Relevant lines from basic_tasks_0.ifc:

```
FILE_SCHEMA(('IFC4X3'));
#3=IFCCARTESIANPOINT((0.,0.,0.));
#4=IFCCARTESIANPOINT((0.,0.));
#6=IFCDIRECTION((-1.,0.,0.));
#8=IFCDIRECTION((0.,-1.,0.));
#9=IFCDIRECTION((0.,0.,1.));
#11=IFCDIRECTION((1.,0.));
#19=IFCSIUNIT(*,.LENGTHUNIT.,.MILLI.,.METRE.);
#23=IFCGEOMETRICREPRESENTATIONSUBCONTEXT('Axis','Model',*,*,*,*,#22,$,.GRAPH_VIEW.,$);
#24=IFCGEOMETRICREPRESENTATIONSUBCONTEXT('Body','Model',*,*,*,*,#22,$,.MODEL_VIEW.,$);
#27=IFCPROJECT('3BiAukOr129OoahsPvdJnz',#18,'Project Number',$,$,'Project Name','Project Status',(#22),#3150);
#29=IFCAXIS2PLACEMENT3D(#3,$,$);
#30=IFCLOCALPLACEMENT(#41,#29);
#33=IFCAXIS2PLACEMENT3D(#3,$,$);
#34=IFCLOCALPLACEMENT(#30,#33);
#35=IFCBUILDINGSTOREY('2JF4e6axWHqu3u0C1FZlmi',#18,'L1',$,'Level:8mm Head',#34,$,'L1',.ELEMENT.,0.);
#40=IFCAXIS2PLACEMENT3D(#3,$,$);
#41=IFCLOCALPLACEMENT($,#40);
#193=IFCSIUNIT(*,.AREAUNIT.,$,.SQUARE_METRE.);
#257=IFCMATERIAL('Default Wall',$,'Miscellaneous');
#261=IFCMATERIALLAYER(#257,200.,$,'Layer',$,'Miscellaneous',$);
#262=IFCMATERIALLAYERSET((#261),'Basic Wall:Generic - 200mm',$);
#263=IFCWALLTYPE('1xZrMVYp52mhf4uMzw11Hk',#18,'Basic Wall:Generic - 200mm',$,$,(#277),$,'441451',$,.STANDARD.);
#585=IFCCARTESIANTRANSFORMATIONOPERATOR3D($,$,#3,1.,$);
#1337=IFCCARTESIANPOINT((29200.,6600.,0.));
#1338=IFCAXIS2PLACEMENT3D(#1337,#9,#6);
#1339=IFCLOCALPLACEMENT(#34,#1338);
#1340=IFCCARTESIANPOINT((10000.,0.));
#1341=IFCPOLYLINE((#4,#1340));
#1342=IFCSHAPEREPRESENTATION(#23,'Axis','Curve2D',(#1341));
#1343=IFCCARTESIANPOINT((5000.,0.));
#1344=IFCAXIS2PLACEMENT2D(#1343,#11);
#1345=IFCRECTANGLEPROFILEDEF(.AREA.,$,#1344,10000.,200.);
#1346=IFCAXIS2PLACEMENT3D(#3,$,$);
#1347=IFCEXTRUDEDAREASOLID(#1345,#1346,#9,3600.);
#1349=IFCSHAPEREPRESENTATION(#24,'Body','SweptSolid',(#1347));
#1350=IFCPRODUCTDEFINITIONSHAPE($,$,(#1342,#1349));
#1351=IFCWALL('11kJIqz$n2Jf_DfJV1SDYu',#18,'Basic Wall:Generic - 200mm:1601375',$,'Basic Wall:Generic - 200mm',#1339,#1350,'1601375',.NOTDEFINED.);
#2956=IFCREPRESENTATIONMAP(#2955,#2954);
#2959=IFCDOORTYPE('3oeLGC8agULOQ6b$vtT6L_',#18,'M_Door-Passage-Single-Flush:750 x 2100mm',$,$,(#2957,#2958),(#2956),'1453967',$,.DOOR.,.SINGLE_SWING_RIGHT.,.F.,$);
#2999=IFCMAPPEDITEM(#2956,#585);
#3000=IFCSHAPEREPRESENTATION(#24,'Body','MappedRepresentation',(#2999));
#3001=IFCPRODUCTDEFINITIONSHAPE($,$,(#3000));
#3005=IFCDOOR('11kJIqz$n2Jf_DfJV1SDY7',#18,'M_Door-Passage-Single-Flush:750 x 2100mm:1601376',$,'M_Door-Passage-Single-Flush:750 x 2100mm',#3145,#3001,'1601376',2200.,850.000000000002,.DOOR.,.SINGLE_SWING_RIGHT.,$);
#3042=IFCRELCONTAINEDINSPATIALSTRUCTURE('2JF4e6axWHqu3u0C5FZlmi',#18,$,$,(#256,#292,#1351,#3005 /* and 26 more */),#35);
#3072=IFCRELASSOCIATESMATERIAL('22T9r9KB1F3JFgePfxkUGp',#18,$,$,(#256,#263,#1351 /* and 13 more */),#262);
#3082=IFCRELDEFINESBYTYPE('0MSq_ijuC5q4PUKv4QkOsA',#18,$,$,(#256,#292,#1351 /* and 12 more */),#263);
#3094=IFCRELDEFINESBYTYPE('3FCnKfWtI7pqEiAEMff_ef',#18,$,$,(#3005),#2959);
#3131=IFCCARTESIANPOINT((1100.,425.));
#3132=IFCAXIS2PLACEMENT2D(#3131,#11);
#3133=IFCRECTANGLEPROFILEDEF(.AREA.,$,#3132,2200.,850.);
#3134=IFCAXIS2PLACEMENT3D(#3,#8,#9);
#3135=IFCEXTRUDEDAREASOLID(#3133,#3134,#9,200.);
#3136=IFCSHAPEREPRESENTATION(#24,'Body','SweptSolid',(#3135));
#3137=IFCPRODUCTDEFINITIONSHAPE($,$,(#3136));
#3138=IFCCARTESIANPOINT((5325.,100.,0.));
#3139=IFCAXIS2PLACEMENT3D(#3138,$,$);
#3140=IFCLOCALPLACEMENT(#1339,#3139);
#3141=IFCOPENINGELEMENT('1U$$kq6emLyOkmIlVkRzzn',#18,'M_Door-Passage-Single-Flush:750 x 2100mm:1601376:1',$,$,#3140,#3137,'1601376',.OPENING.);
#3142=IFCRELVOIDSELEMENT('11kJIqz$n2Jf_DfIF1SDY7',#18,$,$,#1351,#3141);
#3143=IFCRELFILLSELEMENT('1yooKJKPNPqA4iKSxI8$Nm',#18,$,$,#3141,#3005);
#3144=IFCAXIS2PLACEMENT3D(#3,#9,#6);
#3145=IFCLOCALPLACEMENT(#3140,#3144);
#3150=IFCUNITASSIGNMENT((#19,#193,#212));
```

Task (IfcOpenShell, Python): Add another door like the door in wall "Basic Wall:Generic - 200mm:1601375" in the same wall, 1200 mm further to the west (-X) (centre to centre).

```python
import ifcopenshell
import ifcopenshell.api.feature
import ifcopenshell.api.geometry
import ifcopenshell.api.root
import ifcopenshell.geom
import ifcopenshell.util.element
import ifcopenshell.util.placement
import ifcopenshell.util.shape
import ifcopenshell.util.unit

model = ifcopenshell.open("basic_tasks_0.ifc")
unit_scale = ifcopenshell.util.unit.calculate_unit_scale(model)
settings = ifcopenshell.geom.settings()


def volume(element):
    """Net volume in cubic metres, openings subtracted."""
    shape = ifcopenshell.geom.create_shape(settings, element)
    return ifcopenshell.util.shape.get_volume(shape.geometry)


def reuse_history(source, copy):
    """copy_class also copies each property set's owner history, people and application; keep the originals."""
    for rel in copy.IsDefinedBy:
        if rel.is_a("IfcRelDefinesByProperties") and (history := rel.RelatingPropertyDefinition.OwnerHistory):
            rel.RelatingPropertyDefinition.OwnerHistory = source.OwnerHistory
            ifcopenshell.util.element.remove_deep2(model, history)


door = model.by_guid("11kJIqz$n2Jf_DfJV1SDY7")
opening = door.FillsVoids[0].RelatingOpeningElement
wall = opening.VoidsElements[0].RelatingBuildingElement
before = volume(wall)
shift = ifcopenshell.util.placement.get_local_placement(wall.ObjectPlacement)[:3, 0] * 1.2 / unit_scale

# copy_class copies the void relationship, type, container and properties, but no geometry.
new_opening = ifcopenshell.api.root.copy_class(model, product=opening)
new_opening.Representation = ifcopenshell.util.element.copy_deep(
    model, opening.Representation, exclude=["IfcGeometricRepresentationContext", "IfcRepresentationMap"]
)
new_opening.Name = "M_Door-Passage-Single-Flush:750 x 2100mm"
new_opening.Tag = None
new_door = ifcopenshell.api.root.copy_class(model, product=door)
new_door.Representation = ifcopenshell.util.element.copy_deep(
    model, door.Representation, exclude=["IfcGeometricRepresentationContext", "IfcRepresentationMap"]
)
new_door.Name = "M_Door-Passage-Single-Flush:750 x 2100mm"
new_door.Tag = None
reuse_history(door, new_door)
ifcopenshell.api.feature.add_filling(model, opening=new_opening, element=new_door)

for old, new in ((opening, new_opening), (door, new_door)):
    matrix = ifcopenshell.util.placement.get_local_placement(old.ObjectPlacement)
    matrix[:3, 3] += shift
    ifcopenshell.api.geometry.edit_object_placement(model, product=new, matrix=matrix, is_si=False)

after = volume(wall)

print(f"wall volume {before:.3f} -> {after:.3f} m3")

model.write("basic_tasks_0-out.ifc")
```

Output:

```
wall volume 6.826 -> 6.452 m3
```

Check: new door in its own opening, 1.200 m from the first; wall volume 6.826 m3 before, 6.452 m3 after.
